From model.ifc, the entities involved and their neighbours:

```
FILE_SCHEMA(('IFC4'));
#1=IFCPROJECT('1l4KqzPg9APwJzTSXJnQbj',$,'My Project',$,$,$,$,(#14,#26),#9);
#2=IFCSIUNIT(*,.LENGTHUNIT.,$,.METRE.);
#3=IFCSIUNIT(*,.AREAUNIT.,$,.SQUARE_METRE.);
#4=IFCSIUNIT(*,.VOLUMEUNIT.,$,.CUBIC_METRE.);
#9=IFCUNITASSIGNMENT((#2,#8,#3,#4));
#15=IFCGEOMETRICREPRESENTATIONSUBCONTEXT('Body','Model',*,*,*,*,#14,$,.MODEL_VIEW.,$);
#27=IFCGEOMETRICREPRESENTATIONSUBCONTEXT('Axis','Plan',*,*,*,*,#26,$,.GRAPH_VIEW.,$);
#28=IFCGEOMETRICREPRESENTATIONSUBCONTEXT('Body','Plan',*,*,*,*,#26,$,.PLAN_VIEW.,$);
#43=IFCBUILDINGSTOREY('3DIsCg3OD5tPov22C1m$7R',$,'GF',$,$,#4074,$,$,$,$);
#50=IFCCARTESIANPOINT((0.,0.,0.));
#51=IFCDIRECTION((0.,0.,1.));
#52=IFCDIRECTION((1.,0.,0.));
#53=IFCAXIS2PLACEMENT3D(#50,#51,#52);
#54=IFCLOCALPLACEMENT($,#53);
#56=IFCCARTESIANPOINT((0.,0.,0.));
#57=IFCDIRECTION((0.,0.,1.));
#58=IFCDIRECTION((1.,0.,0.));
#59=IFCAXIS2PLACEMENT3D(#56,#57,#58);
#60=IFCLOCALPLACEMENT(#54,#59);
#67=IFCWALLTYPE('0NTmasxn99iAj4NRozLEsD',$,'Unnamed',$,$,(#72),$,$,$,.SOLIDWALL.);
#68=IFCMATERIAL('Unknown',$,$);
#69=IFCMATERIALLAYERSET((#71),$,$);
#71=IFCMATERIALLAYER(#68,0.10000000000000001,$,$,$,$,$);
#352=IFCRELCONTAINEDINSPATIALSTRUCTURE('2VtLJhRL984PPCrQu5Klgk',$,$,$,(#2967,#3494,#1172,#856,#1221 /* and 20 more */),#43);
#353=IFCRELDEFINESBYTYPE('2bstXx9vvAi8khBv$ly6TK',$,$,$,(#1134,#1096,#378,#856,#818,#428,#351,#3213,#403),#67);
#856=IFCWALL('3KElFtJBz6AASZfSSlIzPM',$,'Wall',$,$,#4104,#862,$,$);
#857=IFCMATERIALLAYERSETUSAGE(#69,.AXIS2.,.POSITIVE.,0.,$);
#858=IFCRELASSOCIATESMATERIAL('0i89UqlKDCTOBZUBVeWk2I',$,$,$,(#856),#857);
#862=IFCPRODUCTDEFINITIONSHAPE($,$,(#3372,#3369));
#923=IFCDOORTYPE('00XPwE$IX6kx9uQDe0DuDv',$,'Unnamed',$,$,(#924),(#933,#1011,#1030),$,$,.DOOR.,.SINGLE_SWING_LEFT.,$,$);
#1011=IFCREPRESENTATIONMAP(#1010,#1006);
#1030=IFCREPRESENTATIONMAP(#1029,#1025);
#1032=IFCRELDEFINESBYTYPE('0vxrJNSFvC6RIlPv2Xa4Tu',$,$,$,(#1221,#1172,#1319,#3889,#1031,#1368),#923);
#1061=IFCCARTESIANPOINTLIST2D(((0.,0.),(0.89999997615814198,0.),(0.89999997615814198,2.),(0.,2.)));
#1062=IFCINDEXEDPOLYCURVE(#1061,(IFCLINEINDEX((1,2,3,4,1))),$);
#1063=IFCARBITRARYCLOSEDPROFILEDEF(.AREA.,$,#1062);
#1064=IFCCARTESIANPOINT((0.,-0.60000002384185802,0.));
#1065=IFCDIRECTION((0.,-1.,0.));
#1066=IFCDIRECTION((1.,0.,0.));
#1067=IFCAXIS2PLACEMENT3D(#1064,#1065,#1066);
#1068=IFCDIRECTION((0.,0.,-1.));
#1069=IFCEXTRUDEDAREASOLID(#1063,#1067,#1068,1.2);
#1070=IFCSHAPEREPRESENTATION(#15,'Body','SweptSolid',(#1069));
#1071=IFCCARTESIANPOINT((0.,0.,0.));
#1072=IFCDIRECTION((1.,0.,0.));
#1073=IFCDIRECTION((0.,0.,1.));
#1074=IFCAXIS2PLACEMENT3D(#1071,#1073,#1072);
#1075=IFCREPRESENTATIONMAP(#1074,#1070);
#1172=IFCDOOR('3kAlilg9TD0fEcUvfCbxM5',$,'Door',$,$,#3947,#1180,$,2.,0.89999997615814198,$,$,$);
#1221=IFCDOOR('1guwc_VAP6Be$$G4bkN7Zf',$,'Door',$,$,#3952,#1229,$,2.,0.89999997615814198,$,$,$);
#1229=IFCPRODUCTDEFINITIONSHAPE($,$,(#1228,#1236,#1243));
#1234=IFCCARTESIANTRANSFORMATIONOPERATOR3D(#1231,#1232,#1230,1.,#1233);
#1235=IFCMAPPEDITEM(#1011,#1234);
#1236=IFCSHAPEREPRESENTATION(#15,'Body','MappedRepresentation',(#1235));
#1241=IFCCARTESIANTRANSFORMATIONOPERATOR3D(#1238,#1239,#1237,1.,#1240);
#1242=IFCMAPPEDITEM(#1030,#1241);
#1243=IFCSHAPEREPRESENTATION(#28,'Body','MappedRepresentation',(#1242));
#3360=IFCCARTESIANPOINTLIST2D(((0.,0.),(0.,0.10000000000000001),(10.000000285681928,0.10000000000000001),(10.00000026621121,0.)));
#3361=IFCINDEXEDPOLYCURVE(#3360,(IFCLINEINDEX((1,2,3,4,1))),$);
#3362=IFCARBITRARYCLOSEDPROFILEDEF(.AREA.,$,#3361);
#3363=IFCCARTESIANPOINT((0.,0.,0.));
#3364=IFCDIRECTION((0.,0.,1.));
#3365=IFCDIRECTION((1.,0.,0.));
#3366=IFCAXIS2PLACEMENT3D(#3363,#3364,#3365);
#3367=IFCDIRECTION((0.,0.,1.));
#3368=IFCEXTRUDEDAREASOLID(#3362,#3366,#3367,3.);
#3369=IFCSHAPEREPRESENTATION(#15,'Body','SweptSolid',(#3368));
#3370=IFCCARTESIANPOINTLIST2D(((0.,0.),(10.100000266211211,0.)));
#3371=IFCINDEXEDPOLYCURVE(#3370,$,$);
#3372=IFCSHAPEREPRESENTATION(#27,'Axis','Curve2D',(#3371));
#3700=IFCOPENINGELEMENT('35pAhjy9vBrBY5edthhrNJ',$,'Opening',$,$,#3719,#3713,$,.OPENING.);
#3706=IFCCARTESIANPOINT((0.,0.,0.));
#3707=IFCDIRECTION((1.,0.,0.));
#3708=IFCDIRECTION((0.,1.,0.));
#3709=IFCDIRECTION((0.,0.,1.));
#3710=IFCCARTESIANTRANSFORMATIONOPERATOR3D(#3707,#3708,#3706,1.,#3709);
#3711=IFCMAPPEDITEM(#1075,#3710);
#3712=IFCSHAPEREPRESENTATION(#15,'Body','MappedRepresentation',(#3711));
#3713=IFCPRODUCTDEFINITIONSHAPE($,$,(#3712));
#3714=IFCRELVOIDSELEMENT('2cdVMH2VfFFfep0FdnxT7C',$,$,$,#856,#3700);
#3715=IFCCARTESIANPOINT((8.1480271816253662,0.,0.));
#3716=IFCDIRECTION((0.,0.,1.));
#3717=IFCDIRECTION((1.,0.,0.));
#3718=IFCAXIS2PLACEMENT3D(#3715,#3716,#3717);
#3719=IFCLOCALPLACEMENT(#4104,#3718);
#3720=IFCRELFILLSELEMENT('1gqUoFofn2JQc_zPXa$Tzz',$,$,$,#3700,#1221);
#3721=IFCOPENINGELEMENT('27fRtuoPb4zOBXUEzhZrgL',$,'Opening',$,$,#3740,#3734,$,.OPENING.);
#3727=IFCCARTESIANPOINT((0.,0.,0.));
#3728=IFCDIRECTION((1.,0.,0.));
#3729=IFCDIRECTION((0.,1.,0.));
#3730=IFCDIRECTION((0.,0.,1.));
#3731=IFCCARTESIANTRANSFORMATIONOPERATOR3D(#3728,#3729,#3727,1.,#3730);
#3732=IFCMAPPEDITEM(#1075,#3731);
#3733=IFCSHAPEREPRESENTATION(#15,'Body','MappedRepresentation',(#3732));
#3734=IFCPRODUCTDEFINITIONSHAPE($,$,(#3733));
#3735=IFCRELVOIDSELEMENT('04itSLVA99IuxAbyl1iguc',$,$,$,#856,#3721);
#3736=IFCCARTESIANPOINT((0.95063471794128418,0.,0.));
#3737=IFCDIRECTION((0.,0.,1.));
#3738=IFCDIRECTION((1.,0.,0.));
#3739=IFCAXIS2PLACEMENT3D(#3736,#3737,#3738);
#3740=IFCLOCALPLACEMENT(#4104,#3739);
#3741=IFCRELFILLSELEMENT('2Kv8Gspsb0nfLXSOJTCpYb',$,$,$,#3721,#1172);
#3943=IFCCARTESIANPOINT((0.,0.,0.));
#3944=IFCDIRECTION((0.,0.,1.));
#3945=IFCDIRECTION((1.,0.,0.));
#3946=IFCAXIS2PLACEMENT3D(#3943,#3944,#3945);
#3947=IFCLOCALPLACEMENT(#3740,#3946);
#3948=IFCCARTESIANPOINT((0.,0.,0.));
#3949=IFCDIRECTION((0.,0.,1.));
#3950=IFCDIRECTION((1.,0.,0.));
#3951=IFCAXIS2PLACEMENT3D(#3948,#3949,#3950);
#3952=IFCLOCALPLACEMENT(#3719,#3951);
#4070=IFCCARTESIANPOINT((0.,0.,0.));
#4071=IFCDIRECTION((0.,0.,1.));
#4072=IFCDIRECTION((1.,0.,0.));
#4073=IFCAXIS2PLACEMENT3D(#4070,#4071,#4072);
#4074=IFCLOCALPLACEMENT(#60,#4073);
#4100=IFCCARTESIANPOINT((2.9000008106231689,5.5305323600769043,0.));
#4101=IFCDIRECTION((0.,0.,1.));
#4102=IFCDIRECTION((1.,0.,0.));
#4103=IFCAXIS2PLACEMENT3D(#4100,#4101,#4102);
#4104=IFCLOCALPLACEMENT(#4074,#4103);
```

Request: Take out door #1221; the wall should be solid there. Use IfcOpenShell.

```python
import ifcopenshell
import ifcopenshell.api.feature
import ifcopenshell.api.root
import ifcopenshell.geom
import ifcopenshell.util.shape

model = ifcopenshell.open("model.ifc")
settings = ifcopenshell.geom.settings()


def volume(element):
    """Net volume in cubic metres, openings subtracted."""
    shape = ifcopenshell.geom.create_shape(settings, element)
    return ifcopenshell.util.shape.get_volume(shape.geometry)


door = model.by_id(1221)
opening = door.FillsVoids[0].RelatingOpeningElement
wall = opening.VoidsElements[0].RelatingBuildingElement
before = volume(wall)

ifcopenshell.api.root.remove_product(model, product=door)
ifcopenshell.api.feature.remove_feature(model, feature=opening)

after = volume(wall)

print(f"wall volume {before:.3f} -> {after:.3f} m3")

model.write("model_edited.ifc")
```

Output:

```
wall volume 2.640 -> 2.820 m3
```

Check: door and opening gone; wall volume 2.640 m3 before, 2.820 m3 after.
